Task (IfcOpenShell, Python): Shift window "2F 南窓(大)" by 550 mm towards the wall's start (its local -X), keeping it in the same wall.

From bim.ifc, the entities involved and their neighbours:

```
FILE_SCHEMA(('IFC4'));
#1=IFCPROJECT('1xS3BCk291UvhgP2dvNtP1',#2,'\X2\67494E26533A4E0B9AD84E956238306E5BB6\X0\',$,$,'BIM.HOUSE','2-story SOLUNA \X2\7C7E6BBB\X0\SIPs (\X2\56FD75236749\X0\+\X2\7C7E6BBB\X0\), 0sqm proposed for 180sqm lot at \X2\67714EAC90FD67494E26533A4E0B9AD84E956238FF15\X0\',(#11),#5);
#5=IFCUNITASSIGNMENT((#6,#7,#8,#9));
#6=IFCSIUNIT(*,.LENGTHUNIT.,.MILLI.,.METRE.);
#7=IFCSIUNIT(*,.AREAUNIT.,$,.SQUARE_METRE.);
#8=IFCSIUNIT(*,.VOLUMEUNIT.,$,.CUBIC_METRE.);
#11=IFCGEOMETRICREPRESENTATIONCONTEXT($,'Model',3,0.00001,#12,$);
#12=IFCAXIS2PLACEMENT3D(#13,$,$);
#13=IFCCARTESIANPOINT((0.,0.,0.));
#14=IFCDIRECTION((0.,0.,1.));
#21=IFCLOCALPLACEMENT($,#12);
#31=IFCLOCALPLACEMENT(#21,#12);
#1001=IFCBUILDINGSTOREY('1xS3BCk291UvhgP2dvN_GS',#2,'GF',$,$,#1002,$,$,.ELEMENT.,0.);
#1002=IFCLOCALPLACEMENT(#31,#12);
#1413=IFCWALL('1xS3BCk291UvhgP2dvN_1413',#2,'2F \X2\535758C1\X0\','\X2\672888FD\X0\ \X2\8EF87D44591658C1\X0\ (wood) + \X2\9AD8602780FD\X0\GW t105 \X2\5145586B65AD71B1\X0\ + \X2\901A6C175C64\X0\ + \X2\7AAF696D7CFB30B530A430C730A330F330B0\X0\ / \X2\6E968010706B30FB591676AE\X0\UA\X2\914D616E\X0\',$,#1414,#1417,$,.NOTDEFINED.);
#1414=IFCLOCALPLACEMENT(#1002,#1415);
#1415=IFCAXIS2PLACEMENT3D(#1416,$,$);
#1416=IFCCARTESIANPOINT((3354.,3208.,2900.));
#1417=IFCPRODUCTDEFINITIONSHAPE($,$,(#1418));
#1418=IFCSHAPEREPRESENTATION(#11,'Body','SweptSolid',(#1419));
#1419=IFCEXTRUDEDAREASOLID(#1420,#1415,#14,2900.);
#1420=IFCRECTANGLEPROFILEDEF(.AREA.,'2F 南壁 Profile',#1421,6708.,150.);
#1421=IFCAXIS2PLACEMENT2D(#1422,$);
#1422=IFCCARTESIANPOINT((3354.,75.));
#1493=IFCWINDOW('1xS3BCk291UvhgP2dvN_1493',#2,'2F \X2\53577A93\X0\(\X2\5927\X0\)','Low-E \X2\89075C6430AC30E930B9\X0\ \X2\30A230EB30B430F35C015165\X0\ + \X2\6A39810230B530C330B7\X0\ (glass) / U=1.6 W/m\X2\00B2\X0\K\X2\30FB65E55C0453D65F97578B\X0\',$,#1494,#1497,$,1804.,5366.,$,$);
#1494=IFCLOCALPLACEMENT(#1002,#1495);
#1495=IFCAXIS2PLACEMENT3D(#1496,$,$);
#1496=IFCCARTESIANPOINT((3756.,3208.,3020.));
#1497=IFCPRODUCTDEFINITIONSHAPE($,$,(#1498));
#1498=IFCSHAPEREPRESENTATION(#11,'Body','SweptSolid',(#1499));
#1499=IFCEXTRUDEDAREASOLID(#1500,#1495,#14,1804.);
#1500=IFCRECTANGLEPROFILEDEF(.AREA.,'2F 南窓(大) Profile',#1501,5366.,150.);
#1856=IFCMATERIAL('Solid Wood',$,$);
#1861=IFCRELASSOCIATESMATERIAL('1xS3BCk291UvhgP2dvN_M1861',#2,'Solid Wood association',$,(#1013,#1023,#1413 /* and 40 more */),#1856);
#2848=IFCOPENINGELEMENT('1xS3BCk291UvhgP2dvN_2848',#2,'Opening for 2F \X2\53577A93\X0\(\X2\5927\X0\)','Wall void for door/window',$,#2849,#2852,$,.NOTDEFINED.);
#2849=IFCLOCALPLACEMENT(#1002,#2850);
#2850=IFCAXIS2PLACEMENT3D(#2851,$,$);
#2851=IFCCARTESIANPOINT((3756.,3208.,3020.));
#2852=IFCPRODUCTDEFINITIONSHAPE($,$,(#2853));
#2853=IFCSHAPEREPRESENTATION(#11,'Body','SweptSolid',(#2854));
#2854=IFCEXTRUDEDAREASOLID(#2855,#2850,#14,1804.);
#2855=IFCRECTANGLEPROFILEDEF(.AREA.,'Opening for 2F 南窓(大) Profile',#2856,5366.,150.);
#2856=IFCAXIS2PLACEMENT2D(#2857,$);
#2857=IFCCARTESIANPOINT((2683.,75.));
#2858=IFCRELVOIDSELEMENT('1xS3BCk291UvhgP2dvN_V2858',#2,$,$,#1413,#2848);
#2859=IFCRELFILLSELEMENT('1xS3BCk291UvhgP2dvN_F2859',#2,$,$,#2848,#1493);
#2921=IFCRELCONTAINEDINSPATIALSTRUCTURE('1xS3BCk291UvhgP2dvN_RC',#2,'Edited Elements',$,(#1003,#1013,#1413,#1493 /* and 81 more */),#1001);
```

```python
import ifcopenshell
import ifcopenshell.api.geometry
import ifcopenshell.util.placement

model = ifcopenshell.open("bim.ifc")

window = model.by_guid("1xS3BCk291UvhgP2dvN_1493")
opening = window.FillsVoids[0].RelatingOpeningElement
wall = opening.VoidsElements[0].RelatingBuildingElement

wall_matrix = ifcopenshell.util.placement.get_local_placement(wall.ObjectPlacement)
shift = wall_matrix[:3, 0] * -550.0
before = ifcopenshell.util.placement.get_local_placement(window.ObjectPlacement)[:3, 3].copy()

# The window is not placed relative to its opening, so move both.
for product in (opening, window):
    matrix = ifcopenshell.util.placement.get_local_placement(product.ObjectPlacement)
    matrix[:3, 3] += shift
    ifcopenshell.api.geometry.edit_object_placement(model, product=product, matrix=matrix, is_si=False)

after = ifcopenshell.util.placement.get_local_placement(window.ObjectPlacement)[:3, 3]
print("window moved by", (after - before).round(3) + 0.0)

model.write("bim_v2.ifc")
```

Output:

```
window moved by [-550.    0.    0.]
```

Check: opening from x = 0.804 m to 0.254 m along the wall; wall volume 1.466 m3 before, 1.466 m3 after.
